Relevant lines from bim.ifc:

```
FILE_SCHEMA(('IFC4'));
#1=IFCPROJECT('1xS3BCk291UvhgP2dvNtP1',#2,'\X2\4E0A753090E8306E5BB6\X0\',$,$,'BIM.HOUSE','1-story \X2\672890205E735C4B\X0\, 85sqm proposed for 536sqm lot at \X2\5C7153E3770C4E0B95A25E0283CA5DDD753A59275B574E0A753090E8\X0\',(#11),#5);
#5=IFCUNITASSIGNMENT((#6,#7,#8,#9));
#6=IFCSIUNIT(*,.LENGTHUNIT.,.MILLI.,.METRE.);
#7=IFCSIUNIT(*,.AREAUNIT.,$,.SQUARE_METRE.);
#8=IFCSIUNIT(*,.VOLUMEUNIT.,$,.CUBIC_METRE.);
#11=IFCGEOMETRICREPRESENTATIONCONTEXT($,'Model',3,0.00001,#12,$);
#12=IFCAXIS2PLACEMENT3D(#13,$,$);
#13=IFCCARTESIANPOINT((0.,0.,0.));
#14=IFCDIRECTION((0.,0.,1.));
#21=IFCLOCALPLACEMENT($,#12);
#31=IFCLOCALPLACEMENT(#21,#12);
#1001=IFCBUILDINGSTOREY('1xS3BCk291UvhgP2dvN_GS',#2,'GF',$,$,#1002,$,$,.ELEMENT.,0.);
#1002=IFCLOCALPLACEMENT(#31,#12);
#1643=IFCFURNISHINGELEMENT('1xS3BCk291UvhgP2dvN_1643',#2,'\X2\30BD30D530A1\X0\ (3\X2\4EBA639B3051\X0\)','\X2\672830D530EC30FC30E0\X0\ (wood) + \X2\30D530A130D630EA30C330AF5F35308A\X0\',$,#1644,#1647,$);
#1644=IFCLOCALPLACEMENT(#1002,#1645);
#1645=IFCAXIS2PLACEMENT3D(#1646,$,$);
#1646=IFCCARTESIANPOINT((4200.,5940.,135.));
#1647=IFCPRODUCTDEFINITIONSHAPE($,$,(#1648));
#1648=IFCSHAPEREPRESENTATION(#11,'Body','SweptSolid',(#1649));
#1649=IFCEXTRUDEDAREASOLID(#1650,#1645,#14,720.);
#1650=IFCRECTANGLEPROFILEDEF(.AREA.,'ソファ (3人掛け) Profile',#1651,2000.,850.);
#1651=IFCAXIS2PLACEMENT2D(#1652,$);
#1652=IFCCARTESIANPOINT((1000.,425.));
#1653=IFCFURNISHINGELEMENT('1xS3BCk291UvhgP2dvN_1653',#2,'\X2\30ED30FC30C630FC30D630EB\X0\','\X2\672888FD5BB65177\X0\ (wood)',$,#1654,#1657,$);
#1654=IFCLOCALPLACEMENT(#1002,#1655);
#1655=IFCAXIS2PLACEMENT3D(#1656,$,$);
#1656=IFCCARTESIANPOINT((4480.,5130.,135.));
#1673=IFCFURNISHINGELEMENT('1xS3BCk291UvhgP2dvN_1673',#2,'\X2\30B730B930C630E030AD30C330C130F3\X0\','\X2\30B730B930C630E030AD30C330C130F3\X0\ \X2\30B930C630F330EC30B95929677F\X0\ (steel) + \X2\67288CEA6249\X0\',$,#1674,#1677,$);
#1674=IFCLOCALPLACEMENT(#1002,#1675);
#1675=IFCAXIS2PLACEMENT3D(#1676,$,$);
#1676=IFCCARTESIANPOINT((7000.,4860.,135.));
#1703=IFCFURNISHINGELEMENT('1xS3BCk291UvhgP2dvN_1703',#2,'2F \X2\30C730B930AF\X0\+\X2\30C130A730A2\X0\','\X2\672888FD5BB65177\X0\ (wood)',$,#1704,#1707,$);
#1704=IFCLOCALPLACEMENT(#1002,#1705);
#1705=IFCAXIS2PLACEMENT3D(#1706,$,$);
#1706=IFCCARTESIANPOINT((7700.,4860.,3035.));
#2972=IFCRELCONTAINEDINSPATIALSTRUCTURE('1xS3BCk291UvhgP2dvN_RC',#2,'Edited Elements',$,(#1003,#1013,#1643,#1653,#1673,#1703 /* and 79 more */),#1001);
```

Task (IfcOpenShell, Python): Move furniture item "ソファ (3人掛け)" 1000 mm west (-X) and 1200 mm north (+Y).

```python
import ifcopenshell
import ifcopenshell.api.geometry
import ifcopenshell.util.placement
import ifcopenshell.util.unit

model = ifcopenshell.open("bim.ifc")
unit_scale = ifcopenshell.util.unit.calculate_unit_scale(model)

item = model.by_guid("1xS3BCk291UvhgP2dvN_1643")
matrix = ifcopenshell.util.placement.get_local_placement(item.ObjectPlacement)
matrix[0, 3] -= 1 / unit_scale
matrix[1, 3] += 1.2 / unit_scale
ifcopenshell.api.geometry.edit_object_placement(model, product=item, matrix=matrix, is_si=False)

print(ifcopenshell.util.placement.get_local_placement(item.ObjectPlacement).round(3) + 0.0)

model.write("bim_v2.ifc")
```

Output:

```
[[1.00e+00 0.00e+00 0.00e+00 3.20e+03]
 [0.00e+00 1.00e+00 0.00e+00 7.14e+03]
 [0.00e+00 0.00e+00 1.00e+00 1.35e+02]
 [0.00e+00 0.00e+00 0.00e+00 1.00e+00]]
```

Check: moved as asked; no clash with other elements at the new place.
